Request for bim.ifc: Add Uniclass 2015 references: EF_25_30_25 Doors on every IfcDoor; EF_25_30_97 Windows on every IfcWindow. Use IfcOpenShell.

First a look at what the model holds.

```python
import ifcopenshell

model = ifcopenshell.open("bim.ifc")
print(model.schema)
print("classifications:", [c.Name for c in model.by_type("IfcClassification")])
for ifc_class in ("IfcDoor", "IfcRoof", "IfcStair", "IfcWall", "IfcWindow"):
    print(ifc_class, len(model.by_type(ifc_class)))
```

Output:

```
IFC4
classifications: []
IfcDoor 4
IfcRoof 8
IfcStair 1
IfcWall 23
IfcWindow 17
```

```python
import ifcopenshell
import ifcopenshell.api.classification

model = ifcopenshell.open("bim.ifc")

system = ifcopenshell.api.classification.add_classification(model, classification="Uniclass 2015")

codes = {
    "IfcDoor": ("EF_25_30_25", "Doors"),
    "IfcWindow": ("EF_25_30_97", "Windows"),
}
for ifc_class, (code, name) in codes.items():
    products = model.by_type(ifc_class)
    ifcopenshell.api.classification.add_reference(
        model, products=products, classification=system, identification=code, name=name
    )
    print(code, len(products))

model.write("bim_v2.ifc")
```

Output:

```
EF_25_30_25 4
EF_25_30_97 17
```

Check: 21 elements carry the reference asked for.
